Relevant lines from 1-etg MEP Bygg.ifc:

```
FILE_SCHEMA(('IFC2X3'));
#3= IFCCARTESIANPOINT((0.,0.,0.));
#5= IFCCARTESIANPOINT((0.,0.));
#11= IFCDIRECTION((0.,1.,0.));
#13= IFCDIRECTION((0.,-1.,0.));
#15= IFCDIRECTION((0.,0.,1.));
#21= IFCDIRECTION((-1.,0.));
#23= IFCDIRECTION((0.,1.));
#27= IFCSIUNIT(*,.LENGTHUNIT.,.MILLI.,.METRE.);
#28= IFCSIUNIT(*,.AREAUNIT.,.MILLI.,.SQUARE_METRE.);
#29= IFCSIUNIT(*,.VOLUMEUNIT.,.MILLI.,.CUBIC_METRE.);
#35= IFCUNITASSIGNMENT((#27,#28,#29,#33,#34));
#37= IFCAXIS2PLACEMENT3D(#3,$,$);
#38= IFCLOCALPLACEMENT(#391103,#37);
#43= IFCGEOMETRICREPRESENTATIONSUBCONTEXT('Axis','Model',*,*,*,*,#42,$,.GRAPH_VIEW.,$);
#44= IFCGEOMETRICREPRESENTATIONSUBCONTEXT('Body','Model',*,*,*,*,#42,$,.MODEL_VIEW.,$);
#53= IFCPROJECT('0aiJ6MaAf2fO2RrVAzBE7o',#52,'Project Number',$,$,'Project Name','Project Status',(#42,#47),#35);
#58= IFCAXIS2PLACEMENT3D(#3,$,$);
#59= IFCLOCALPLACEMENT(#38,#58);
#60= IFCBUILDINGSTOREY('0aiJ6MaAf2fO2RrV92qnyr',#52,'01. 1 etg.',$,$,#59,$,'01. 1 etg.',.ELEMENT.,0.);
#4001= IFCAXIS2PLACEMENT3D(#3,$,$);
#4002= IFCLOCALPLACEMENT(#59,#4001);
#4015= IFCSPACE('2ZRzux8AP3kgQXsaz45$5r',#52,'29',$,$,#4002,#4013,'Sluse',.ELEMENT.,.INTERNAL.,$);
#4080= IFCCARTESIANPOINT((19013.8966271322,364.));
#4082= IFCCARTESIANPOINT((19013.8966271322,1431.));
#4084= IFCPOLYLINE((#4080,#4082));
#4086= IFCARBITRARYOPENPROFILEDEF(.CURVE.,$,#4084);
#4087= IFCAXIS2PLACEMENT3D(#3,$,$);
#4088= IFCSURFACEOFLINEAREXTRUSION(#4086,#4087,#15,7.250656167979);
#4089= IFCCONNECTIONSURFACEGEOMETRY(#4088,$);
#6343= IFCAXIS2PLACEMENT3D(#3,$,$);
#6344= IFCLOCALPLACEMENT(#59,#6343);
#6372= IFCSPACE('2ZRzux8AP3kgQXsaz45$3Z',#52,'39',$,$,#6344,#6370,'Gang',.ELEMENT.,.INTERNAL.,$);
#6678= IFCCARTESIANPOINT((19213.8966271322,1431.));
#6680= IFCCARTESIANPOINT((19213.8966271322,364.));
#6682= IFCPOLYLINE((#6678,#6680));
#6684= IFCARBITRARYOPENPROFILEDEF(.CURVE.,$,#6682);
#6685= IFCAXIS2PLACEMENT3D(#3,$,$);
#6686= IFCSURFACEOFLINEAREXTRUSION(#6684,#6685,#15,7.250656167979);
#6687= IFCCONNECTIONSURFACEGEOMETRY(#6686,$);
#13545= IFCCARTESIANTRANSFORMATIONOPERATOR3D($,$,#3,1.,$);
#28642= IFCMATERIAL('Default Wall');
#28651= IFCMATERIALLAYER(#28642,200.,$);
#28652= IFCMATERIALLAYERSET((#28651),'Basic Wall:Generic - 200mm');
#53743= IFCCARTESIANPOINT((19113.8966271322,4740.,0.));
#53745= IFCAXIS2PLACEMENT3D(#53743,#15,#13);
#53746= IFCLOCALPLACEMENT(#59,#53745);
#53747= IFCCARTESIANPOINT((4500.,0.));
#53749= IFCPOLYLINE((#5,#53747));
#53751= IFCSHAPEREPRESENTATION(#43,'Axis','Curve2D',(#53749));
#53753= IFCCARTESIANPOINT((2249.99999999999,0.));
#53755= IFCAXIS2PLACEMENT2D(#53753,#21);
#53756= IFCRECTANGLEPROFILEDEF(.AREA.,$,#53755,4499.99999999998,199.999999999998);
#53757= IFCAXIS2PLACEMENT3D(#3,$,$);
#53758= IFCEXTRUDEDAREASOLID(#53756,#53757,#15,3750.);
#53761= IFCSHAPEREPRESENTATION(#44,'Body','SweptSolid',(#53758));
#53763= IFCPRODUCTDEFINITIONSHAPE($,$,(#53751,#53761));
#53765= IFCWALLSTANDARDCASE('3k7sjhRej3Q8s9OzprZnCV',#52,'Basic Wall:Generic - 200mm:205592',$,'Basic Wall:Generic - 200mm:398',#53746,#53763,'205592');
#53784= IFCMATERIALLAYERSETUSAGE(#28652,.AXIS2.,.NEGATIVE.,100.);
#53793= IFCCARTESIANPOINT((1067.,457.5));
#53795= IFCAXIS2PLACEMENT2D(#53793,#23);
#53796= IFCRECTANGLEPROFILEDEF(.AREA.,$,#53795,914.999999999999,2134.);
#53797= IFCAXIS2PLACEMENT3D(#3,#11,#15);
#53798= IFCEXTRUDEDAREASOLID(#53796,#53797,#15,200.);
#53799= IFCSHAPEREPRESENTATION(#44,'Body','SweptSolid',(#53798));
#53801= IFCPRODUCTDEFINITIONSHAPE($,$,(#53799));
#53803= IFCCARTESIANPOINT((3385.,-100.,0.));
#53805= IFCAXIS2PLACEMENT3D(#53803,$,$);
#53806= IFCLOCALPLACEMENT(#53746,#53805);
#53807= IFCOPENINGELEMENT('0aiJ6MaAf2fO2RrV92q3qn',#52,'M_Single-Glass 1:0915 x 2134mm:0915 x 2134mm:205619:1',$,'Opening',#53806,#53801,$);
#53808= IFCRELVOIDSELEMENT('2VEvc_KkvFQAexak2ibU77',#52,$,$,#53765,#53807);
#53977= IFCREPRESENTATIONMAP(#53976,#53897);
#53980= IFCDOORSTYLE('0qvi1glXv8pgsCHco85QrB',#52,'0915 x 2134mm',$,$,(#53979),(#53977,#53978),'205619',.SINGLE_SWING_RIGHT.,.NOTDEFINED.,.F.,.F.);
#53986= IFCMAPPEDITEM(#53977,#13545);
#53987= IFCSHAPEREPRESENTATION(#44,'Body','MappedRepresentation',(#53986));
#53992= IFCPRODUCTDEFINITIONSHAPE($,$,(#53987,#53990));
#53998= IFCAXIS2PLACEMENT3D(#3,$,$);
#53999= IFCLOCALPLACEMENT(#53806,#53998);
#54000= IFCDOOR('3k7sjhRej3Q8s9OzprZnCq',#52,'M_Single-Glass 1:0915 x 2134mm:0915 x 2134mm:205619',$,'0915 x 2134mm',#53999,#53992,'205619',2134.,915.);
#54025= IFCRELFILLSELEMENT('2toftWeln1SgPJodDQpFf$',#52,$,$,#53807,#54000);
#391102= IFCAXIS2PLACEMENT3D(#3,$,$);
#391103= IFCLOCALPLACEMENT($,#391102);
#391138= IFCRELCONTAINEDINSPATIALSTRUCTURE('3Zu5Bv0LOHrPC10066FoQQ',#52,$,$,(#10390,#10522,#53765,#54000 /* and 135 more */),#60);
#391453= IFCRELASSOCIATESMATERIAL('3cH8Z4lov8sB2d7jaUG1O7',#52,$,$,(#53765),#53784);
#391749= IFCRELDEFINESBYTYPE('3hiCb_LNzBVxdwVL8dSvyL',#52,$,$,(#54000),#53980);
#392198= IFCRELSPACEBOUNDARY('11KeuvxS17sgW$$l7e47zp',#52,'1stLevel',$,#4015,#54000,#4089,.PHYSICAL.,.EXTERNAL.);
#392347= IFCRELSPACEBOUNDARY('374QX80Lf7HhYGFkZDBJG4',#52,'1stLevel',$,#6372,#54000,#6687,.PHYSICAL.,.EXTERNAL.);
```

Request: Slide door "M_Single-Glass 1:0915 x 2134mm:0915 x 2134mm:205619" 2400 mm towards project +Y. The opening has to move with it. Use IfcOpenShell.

```python
import numpy as np
import ifcopenshell
import ifcopenshell.api.geometry
import ifcopenshell.util.placement

model = ifcopenshell.open("1-etg MEP Bygg.ifc")

door = model.by_id(54000)
opening = door.FillsVoids[0].RelatingOpeningElement
wall = opening.VoidsElements[0].RelatingBuildingElement

wall_matrix = ifcopenshell.util.placement.get_local_placement(wall.ObjectPlacement)
shift = wall_matrix[:3, 0] * -2400.0
before = ifcopenshell.util.placement.get_local_placement(door.ObjectPlacement)[:3, 3].copy()

# The door is placed relative to its opening, so it follows when the opening moves.
matrix = ifcopenshell.util.placement.get_local_placement(opening.ObjectPlacement)
matrix[:3, 3] += shift
ifcopenshell.api.geometry.edit_object_placement(
    model, product=opening, matrix=matrix, is_si=False, should_transform_children=True
)

# Space boundary surfaces are stored in each space's coordinates; move them too.
for rel in door.ProvidesBoundaries:
    if not rel.ConnectionGeometry:
        continue
    surface = rel.ConnectionGeometry.SurfaceOnRelatingElement
    space_matrix = ifcopenshell.util.placement.get_local_placement(rel.RelatingSpace.ObjectPlacement)
    point = np.array(surface.Position.Location.Coordinates) + space_matrix[:3, :3].T @ shift
    surface.Position = model.createIfcAxis2Placement3D(
        model.createIfcCartesianPoint(point.tolist()), surface.Position.Axis, surface.Position.RefDirection
    )

after = ifcopenshell.util.placement.get_local_placement(door.ObjectPlacement)[:3, 3]
print("door moved by", (after - before).round(3) + 0.0)

model.write("1-etg MEP Bygg-out.ifc")
```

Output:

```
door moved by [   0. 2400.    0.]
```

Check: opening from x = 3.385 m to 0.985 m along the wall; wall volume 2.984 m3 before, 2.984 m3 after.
